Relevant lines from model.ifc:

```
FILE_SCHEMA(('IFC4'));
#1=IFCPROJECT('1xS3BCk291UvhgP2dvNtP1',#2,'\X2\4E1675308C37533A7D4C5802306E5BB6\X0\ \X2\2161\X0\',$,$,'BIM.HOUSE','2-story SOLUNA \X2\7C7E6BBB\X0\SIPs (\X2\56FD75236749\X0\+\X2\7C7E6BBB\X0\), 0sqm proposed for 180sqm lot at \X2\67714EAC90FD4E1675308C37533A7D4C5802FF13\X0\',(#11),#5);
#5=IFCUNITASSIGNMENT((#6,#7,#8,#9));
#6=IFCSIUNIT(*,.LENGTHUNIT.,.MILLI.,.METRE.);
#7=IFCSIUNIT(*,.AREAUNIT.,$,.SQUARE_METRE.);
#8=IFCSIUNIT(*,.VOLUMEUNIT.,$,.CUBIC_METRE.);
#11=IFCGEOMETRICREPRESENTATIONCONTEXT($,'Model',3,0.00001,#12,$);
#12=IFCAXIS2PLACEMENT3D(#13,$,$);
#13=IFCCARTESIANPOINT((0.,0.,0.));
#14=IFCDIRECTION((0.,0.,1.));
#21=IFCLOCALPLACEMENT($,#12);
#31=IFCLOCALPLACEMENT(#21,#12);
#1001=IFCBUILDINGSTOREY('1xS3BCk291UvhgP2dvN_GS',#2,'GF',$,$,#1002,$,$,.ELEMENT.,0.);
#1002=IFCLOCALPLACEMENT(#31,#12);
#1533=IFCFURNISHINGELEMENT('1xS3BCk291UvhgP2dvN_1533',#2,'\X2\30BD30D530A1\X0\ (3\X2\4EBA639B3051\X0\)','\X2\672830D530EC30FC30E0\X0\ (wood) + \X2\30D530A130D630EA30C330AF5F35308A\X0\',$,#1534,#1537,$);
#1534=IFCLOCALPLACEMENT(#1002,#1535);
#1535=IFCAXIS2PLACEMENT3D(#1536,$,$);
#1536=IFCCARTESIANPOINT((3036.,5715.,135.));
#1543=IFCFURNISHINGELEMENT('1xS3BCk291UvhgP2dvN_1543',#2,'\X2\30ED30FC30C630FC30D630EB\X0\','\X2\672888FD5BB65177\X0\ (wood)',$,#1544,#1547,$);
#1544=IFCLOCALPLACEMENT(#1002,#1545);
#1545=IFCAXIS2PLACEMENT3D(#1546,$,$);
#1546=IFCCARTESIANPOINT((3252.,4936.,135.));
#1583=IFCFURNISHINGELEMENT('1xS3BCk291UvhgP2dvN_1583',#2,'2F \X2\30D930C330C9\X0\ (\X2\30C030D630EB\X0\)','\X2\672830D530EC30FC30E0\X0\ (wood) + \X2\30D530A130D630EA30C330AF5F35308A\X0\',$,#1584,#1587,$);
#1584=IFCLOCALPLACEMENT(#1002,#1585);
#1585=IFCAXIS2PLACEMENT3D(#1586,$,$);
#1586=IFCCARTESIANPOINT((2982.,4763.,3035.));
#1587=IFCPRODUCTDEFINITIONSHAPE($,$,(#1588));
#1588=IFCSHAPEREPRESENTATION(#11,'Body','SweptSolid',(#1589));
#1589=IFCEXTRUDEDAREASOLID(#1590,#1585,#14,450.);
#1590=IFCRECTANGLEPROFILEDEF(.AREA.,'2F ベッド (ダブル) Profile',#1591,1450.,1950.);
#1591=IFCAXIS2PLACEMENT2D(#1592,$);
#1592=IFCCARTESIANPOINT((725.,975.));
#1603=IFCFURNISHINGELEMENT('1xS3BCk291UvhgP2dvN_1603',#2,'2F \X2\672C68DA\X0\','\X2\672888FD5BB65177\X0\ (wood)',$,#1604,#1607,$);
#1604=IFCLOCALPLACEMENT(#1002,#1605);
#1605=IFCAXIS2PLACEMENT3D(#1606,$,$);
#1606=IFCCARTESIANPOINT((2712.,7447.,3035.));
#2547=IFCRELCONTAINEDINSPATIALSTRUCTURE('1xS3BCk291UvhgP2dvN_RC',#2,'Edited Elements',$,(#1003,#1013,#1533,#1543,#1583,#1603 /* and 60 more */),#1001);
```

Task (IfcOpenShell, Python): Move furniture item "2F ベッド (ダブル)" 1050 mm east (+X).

```python
import ifcopenshell
import ifcopenshell.api.geometry
import ifcopenshell.util.placement
import ifcopenshell.util.unit

model = ifcopenshell.open("model.ifc")
unit_scale = ifcopenshell.util.unit.calculate_unit_scale(model)

item = model.by_guid("1xS3BCk291UvhgP2dvN_1583")
matrix = ifcopenshell.util.placement.get_local_placement(item.ObjectPlacement)
matrix[0, 3] += 1.05 / unit_scale
ifcopenshell.api.geometry.edit_object_placement(model, product=item, matrix=matrix, is_si=False)

print(ifcopenshell.util.placement.get_local_placement(item.ObjectPlacement).round(3) + 0.0)

model.write("model_v2.ifc")
```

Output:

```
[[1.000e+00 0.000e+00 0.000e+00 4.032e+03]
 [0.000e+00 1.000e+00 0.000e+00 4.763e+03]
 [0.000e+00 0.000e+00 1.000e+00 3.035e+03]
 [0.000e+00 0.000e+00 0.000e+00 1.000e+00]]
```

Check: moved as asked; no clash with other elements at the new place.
